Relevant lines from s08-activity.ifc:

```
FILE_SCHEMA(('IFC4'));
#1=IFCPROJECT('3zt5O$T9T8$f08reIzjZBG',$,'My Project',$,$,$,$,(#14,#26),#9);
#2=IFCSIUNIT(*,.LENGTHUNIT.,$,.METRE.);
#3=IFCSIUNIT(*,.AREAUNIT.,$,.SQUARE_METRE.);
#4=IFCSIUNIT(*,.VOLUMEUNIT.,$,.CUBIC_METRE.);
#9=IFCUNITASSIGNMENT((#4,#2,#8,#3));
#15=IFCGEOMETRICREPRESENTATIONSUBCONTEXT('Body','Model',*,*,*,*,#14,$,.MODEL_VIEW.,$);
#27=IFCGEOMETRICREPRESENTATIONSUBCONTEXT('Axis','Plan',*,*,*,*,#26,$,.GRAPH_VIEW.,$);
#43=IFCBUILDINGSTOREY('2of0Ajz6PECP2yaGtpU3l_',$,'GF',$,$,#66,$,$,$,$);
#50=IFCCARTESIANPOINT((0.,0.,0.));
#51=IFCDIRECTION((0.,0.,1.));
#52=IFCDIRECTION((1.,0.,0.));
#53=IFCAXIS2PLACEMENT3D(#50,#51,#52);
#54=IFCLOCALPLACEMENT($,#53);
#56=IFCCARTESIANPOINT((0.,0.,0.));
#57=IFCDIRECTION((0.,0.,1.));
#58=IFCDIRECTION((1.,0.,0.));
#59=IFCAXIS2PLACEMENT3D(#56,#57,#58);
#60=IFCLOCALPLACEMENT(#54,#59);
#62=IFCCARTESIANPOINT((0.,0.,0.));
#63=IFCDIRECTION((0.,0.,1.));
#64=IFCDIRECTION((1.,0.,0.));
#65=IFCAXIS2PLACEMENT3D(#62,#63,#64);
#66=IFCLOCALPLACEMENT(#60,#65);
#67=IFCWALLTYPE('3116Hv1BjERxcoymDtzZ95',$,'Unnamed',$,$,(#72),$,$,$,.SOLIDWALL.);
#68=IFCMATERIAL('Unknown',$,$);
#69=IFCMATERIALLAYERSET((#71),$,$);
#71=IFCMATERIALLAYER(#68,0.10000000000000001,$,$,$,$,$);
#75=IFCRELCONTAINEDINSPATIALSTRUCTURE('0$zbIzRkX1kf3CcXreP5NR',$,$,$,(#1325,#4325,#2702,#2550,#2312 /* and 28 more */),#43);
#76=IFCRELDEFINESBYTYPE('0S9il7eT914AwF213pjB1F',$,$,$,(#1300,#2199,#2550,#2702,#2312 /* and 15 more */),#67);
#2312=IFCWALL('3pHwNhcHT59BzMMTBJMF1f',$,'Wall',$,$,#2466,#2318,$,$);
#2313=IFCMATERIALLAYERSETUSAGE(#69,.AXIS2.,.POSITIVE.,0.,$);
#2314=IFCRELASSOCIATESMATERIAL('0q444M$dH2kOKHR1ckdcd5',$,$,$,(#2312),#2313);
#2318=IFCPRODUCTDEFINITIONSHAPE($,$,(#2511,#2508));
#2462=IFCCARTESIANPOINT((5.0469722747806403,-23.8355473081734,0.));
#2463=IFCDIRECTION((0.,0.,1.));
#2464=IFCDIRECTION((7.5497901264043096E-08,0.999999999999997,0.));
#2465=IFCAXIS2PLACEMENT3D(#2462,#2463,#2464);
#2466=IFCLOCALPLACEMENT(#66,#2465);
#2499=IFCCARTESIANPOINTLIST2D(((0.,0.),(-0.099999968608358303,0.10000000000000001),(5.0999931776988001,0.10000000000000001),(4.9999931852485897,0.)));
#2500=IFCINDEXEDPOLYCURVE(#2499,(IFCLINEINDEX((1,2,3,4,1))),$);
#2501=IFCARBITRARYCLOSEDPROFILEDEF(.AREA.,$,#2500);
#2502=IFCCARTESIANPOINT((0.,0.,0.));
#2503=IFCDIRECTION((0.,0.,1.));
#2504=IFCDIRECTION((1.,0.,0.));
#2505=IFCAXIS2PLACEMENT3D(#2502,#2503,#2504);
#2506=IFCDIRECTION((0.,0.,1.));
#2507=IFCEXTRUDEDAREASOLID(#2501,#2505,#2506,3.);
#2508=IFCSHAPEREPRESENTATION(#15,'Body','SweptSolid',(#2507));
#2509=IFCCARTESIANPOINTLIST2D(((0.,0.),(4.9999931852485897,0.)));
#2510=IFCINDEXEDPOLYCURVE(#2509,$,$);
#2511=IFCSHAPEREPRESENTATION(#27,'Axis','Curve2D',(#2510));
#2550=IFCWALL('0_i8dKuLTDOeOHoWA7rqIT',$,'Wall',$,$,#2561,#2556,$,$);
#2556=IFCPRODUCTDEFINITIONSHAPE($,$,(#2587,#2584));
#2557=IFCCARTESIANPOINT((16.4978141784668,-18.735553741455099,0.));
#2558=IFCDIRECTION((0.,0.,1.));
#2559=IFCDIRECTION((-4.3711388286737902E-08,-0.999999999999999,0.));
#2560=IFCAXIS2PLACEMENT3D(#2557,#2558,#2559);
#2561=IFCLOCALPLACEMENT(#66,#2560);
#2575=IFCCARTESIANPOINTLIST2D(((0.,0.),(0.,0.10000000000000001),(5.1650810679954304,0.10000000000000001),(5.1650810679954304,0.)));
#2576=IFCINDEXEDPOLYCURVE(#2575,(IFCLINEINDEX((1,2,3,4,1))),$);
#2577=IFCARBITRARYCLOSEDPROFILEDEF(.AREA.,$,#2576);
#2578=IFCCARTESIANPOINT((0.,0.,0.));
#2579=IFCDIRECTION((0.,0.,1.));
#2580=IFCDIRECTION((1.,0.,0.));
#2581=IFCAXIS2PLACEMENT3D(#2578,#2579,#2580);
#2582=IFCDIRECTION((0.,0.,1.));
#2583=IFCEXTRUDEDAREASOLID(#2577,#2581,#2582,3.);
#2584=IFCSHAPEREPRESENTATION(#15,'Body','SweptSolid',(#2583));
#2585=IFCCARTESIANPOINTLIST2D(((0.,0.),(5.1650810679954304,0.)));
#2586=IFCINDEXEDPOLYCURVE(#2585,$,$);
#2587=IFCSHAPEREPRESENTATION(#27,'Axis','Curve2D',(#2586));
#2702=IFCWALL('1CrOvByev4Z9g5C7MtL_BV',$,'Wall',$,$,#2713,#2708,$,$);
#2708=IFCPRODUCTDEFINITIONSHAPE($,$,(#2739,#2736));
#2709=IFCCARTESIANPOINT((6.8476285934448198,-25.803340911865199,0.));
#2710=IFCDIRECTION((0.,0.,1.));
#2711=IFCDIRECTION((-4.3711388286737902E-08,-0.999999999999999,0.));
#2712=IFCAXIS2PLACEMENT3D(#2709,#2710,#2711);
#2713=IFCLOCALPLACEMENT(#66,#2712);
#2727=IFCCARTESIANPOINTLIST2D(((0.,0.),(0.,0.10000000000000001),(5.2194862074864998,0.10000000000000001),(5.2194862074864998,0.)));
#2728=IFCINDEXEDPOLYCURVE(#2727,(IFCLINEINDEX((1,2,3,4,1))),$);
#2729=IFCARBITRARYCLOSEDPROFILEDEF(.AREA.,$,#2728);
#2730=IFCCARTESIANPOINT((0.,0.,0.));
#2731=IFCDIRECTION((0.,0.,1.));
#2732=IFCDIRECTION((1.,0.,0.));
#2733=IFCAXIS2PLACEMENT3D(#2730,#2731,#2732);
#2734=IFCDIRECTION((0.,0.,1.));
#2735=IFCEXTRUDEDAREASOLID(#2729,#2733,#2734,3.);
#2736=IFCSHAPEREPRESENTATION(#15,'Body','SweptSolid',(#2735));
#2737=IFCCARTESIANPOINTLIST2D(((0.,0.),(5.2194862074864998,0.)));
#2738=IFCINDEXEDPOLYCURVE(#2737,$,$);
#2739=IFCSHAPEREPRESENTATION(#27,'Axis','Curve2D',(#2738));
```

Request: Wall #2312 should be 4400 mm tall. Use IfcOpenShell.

```python
import ifcopenshell
import ifcopenshell.geom
import ifcopenshell.util.representation
import ifcopenshell.util.shape
import ifcopenshell.util.unit

model = ifcopenshell.open("s08-activity.ifc")
unit_scale = ifcopenshell.util.unit.calculate_unit_scale(model)
settings = ifcopenshell.geom.settings()


def volume(element):
    """Net volume in cubic metres, openings subtracted."""
    shape = ifcopenshell.geom.create_shape(settings, element)
    return ifcopenshell.util.shape.get_volume(shape.geometry)


wall = model.by_guid("3pHwNhcHT59BzMMTBJMF1f")
before = volume(wall)

body = ifcopenshell.util.representation.get_representation(wall, "Model", "Body")
solid = body.Items[0]
old_height = solid.Depth
solid.Depth = 4.4 / unit_scale
after = volume(wall)

print(f"height {old_height:g} -> {solid.Depth:g}, volume {before:.3f} -> {after:.3f} m3")

model.write("s08-activity_edited.ifc")
```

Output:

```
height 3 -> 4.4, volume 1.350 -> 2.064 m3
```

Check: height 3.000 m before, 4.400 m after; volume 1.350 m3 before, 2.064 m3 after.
